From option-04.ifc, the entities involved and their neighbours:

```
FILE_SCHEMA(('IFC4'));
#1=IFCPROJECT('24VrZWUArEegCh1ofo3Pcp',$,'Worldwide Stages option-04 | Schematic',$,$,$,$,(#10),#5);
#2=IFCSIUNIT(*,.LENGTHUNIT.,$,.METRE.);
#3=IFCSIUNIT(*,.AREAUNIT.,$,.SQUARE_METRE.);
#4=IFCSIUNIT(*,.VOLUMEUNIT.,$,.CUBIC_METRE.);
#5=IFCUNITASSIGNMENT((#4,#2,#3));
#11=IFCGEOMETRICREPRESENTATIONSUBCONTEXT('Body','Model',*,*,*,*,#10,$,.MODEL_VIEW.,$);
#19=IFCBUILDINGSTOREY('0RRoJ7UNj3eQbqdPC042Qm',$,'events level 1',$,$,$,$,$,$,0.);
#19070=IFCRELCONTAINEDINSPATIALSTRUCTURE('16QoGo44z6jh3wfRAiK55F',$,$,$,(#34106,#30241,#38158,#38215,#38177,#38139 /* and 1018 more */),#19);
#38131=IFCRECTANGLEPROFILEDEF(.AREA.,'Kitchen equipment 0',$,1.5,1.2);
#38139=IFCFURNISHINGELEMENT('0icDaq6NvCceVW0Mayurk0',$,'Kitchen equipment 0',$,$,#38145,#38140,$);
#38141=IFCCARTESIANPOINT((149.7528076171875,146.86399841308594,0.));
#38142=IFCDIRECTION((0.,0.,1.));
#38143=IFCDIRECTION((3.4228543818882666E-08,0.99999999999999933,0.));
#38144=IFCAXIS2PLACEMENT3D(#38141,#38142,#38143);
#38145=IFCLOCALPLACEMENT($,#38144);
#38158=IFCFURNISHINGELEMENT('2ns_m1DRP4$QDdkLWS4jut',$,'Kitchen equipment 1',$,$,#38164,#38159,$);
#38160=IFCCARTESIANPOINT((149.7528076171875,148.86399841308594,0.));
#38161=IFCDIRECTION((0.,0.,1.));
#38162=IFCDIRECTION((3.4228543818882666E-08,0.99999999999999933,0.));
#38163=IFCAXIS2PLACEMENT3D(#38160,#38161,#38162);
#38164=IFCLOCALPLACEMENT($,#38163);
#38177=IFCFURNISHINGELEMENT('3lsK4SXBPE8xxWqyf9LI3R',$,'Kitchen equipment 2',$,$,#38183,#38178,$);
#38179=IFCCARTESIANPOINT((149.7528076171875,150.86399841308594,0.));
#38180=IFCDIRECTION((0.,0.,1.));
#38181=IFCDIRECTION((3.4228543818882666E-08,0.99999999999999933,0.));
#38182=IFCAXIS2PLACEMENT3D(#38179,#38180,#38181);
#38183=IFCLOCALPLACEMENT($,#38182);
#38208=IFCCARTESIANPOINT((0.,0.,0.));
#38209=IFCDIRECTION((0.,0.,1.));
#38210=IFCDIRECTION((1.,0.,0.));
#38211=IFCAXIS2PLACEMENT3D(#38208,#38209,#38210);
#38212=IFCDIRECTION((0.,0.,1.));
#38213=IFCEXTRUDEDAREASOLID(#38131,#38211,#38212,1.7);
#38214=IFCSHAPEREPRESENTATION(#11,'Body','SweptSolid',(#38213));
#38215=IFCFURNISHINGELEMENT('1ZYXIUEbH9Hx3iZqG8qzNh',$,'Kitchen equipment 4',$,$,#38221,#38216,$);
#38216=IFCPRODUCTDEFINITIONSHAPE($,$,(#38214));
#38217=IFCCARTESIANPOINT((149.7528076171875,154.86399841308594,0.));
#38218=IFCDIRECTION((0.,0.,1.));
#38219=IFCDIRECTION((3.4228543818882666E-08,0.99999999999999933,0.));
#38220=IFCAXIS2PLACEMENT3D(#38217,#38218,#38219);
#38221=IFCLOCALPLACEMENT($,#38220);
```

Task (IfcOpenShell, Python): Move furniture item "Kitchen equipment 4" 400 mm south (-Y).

```python
import ifcopenshell
import ifcopenshell.api.geometry
import ifcopenshell.util.placement

model = ifcopenshell.open("option-04.ifc")

item = model.by_id(38215)
matrix = ifcopenshell.util.placement.get_local_placement(item.ObjectPlacement)
matrix[1, 3] -= 0.4
ifcopenshell.api.geometry.edit_object_placement(model, product=item, matrix=matrix, is_si=False)

print(ifcopenshell.util.placement.get_local_placement(item.ObjectPlacement).round(3) + 0.0)

model.write("option-04_rev.ifc")
```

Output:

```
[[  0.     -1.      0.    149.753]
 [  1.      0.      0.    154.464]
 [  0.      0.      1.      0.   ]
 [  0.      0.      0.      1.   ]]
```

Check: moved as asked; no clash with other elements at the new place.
